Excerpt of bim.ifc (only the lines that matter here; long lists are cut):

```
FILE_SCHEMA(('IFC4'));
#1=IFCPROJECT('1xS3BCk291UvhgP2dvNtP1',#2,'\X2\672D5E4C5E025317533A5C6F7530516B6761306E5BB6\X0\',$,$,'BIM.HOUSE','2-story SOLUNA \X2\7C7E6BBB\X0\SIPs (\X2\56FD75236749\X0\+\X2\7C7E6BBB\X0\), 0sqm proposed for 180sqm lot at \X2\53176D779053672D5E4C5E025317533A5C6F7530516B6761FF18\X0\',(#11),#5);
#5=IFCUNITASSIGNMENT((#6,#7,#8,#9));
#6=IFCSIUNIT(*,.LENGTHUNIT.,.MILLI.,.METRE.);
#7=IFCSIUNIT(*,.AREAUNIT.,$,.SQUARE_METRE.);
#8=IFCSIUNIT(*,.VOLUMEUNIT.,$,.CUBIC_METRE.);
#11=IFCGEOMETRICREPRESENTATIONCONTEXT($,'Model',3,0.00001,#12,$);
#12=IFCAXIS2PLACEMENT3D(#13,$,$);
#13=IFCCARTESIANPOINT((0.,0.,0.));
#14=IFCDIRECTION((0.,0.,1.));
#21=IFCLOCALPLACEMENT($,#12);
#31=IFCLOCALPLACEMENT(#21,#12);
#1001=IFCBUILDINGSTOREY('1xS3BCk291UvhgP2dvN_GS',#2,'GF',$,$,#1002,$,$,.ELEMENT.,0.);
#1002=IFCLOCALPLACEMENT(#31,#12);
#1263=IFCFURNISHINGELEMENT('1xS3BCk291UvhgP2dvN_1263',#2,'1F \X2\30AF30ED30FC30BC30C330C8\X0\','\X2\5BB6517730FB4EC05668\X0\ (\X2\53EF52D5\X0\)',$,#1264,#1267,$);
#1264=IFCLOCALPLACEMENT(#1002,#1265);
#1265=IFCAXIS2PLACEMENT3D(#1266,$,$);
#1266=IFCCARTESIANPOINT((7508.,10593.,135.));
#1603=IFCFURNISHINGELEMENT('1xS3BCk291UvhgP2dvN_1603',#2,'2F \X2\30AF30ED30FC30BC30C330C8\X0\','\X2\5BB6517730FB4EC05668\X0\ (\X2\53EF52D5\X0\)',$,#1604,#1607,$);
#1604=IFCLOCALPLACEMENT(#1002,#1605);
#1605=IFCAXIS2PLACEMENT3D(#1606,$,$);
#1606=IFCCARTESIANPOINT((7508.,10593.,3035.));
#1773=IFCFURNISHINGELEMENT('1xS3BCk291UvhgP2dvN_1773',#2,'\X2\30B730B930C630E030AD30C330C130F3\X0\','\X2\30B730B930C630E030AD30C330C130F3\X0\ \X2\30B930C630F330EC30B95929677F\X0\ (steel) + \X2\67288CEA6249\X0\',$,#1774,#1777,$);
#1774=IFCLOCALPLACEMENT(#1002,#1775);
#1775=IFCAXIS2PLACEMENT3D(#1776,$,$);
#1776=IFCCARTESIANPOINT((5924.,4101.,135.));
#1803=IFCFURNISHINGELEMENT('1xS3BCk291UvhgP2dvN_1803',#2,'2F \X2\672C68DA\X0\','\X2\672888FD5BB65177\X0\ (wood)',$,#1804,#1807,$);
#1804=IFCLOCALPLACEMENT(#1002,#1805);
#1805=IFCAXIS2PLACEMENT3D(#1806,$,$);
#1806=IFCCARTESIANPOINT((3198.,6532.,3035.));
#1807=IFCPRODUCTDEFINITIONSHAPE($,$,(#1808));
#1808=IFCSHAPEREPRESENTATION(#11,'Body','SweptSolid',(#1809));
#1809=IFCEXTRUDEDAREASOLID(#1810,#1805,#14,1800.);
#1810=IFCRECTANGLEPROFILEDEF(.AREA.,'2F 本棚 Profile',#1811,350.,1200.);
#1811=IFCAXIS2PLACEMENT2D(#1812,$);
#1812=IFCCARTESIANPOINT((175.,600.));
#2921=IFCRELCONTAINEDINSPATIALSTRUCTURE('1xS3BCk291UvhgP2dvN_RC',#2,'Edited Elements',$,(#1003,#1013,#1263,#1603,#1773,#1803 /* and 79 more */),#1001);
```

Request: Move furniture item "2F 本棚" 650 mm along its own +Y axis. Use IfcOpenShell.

```python
import ifcopenshell
import ifcopenshell.api.geometry
import ifcopenshell.util.placement
import ifcopenshell.util.unit

model = ifcopenshell.open("bim.ifc")
unit_scale = ifcopenshell.util.unit.calculate_unit_scale(model)

item = model.by_guid("1xS3BCk291UvhgP2dvN_1803")
matrix = ifcopenshell.util.placement.get_local_placement(item.ObjectPlacement)
matrix[:3, 3] += matrix[:3, 1] * 0.65 / unit_scale
ifcopenshell.api.geometry.edit_object_placement(model, product=item, matrix=matrix, is_si=False)

print(ifcopenshell.util.placement.get_local_placement(item.ObjectPlacement).round(3) + 0.0)

model.write("bim_updated.ifc")
```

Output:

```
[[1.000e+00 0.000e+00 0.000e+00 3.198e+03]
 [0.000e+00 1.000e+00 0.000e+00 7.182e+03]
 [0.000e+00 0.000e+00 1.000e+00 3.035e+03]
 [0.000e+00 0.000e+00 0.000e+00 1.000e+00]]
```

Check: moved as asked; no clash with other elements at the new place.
